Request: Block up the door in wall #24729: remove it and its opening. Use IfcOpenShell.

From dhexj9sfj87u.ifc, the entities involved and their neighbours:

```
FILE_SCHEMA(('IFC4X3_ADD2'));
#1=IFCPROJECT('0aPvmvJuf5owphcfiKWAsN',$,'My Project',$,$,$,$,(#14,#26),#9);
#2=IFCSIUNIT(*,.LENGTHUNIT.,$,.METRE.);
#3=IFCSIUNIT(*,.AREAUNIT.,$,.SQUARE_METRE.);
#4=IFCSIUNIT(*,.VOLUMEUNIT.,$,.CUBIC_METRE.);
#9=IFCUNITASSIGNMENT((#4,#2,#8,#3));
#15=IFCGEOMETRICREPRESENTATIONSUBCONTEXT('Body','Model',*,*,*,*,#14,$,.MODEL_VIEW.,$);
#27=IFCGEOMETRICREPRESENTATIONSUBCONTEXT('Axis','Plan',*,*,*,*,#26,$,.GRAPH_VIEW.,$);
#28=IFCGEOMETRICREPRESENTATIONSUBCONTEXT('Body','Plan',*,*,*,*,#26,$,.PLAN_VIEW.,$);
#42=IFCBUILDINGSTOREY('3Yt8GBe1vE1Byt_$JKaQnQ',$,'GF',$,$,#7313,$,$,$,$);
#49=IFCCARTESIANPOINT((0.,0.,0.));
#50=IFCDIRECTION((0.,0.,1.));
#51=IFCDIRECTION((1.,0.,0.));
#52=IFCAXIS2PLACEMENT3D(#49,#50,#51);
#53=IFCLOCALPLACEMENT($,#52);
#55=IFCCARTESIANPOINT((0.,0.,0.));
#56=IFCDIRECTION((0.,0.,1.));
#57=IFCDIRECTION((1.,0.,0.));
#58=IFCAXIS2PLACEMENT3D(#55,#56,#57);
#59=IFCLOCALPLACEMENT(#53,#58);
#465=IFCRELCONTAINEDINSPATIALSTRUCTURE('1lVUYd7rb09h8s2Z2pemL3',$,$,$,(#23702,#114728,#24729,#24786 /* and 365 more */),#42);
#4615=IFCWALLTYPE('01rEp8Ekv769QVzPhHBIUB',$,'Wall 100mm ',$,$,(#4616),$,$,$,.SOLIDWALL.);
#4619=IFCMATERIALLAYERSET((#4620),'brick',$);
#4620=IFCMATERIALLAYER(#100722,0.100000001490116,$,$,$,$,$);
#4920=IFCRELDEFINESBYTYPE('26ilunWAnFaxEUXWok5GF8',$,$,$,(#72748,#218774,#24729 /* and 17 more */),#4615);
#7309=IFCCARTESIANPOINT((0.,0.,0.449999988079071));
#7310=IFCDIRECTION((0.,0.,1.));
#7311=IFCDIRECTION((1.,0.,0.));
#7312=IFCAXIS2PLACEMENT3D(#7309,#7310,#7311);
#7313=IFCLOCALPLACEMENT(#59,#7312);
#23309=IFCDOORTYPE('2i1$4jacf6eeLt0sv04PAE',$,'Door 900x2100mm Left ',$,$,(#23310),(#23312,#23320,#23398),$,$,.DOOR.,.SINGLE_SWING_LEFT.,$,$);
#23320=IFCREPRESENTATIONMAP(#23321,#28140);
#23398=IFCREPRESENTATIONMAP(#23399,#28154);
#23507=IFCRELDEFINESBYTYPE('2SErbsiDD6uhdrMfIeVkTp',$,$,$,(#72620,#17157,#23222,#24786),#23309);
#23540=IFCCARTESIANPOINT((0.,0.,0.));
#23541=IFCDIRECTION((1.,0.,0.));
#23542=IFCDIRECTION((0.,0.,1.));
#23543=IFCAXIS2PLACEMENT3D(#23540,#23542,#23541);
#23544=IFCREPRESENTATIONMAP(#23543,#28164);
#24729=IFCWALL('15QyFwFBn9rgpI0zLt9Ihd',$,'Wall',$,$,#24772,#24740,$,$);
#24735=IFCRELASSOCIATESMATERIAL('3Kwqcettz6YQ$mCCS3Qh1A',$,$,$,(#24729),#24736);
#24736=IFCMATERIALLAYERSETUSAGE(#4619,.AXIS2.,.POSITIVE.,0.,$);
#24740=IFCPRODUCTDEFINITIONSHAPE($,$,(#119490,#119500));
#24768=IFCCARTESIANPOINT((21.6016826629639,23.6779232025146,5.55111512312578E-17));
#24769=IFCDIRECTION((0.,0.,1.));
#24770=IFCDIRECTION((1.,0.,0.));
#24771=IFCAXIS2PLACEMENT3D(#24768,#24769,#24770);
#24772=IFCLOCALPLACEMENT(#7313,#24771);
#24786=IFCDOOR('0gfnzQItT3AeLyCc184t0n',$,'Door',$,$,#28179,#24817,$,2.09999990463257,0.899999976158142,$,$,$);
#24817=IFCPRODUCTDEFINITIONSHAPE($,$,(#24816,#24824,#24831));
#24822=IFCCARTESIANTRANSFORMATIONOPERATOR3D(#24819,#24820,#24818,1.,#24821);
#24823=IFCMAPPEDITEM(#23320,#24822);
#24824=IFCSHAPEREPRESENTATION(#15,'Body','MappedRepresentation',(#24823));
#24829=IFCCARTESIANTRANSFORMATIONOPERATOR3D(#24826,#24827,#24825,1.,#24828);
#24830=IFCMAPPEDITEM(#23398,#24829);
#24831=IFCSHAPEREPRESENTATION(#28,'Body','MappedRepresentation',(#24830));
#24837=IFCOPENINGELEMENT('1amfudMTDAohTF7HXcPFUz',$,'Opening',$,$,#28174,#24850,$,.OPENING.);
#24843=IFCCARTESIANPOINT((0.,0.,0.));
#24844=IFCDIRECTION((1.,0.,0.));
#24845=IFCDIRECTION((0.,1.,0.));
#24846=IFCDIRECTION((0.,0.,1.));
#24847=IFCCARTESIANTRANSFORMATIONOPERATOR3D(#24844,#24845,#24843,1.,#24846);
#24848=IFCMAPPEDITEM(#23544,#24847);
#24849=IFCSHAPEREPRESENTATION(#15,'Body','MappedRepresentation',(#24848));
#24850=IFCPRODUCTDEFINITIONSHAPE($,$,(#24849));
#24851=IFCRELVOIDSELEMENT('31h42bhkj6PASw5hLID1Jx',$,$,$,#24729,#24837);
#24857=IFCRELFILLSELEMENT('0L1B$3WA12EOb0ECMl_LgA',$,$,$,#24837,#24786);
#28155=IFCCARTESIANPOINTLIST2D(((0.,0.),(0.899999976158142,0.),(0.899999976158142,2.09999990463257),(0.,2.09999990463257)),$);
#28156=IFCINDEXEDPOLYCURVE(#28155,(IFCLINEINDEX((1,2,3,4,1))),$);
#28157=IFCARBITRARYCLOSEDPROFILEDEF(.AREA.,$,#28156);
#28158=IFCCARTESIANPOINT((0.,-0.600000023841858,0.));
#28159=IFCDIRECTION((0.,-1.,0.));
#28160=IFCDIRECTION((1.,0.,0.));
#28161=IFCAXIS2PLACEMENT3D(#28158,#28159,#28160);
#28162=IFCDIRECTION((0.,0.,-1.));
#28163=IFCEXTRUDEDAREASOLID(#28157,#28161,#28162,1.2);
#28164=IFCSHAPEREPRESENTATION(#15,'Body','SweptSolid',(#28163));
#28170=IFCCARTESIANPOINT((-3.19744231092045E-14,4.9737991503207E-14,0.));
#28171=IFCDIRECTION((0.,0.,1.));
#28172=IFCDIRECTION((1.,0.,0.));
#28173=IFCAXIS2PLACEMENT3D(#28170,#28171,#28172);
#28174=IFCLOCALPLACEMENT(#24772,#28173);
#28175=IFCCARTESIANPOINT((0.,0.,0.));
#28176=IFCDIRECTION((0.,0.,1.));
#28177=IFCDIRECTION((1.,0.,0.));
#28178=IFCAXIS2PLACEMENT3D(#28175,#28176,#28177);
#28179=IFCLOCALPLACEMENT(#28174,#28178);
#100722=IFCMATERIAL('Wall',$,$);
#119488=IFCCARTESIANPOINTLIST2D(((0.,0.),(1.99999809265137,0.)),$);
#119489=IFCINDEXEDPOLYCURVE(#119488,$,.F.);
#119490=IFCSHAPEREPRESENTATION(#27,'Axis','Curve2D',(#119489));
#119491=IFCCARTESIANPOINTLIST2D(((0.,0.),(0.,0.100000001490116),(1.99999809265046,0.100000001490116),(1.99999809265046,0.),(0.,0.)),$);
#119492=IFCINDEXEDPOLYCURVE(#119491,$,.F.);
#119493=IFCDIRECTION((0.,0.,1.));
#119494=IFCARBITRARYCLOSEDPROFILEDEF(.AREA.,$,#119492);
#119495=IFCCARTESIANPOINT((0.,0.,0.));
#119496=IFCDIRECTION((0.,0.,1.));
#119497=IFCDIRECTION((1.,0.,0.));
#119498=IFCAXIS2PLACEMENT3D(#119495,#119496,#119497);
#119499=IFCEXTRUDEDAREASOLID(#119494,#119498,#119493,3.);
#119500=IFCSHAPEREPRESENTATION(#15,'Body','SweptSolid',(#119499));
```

```python
import ifcopenshell
import ifcopenshell.api.feature
import ifcopenshell.api.root
import ifcopenshell.geom
import ifcopenshell.util.shape

model = ifcopenshell.open("dhexj9sfj87u.ifc")
settings = ifcopenshell.geom.settings()


def volume(element):
    """Net volume in cubic metres, openings subtracted."""
    shape = ifcopenshell.geom.create_shape(settings, element)
    return ifcopenshell.util.shape.get_volume(shape.geometry)


door = model.by_guid("0gfnzQItT3AeLyCc184t0n")
opening = door.FillsVoids[0].RelatingOpeningElement
wall = opening.VoidsElements[0].RelatingBuildingElement
before = volume(wall)

ifcopenshell.api.root.remove_product(model, product=door)
ifcopenshell.api.feature.remove_feature(model, feature=opening)

after = volume(wall)

print(f"wall volume {before:.3f} -> {after:.3f} m3")

model.write("dhexj9sfj87u_v2.ifc")
```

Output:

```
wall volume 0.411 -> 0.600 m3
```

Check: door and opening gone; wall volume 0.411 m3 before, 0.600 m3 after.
